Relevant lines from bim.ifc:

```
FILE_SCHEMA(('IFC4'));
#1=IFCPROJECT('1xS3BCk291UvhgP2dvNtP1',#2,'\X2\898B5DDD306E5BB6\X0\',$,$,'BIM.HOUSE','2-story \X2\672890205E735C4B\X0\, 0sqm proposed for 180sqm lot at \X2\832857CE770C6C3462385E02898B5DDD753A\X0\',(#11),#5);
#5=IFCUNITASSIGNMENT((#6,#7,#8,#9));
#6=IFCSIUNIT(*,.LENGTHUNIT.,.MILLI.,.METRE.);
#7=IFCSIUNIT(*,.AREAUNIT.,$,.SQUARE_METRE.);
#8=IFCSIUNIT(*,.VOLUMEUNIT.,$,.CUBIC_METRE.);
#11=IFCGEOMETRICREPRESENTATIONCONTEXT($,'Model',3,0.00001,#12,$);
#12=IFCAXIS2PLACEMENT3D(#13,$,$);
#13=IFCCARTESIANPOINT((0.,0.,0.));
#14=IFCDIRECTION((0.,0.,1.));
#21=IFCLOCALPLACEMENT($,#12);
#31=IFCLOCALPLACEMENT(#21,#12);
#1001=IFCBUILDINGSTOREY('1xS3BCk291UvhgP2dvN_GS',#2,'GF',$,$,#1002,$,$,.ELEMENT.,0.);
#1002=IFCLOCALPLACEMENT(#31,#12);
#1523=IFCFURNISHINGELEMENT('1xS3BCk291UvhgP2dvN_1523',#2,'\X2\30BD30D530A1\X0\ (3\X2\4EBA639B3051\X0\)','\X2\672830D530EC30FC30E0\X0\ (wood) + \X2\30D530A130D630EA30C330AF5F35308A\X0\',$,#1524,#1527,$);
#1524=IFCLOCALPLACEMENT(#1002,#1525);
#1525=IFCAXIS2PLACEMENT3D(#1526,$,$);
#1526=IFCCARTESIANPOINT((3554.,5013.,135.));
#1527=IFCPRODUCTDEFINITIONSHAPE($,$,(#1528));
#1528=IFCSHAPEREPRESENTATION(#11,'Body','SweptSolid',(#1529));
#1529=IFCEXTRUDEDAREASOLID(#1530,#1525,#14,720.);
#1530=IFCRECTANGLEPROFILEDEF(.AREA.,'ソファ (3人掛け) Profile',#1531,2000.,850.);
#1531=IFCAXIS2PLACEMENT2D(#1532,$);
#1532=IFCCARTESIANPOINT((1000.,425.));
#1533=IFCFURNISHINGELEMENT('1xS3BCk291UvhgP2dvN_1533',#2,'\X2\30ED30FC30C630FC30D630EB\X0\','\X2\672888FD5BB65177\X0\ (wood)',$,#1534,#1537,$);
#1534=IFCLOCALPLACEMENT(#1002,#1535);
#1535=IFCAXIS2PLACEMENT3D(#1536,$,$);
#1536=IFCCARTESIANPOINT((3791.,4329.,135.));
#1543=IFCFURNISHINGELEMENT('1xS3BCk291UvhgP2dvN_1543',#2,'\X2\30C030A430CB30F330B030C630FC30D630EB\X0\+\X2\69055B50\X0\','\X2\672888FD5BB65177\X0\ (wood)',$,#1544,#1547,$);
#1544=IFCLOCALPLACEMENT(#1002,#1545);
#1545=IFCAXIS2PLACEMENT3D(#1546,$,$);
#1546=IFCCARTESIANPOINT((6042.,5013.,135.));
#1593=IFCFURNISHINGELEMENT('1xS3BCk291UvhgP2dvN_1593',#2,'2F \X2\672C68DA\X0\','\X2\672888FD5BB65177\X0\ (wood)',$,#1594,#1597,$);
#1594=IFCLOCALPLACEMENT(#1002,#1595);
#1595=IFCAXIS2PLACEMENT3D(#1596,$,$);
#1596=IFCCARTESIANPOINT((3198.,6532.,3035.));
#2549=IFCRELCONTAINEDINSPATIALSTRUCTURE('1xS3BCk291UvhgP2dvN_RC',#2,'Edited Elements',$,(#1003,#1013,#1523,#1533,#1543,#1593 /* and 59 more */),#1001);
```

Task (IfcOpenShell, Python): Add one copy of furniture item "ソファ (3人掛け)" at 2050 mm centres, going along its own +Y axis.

```python
import ifcopenshell
import ifcopenshell.api.geometry
import ifcopenshell.api.root
import ifcopenshell.util.element
import ifcopenshell.util.placement
import ifcopenshell.util.unit

model = ifcopenshell.open("bim.ifc")
unit_scale = ifcopenshell.util.unit.calculate_unit_scale(model)


def reuse_history(source, copy):
    """copy_class also copies each property set's owner history, people and application; keep the originals."""
    for rel in copy.IsDefinedBy:
        if rel.is_a("IfcRelDefinesByProperties") and (history := rel.RelatingPropertyDefinition.OwnerHistory):
            rel.RelatingPropertyDefinition.OwnerHistory = source.OwnerHistory
            ifcopenshell.util.element.remove_deep2(model, history)


source = model.by_guid("1xS3BCk291UvhgP2dvN_1523")
base = ifcopenshell.util.placement.get_local_placement(source.ObjectPlacement)
step = base[:3, 1] * 2.05 / unit_scale

for i in range(1, 2):
    copy = ifcopenshell.api.root.copy_class(model, product=source)
    copy.Representation = ifcopenshell.util.element.copy_deep(
        model, source.Representation, exclude=["IfcGeometricRepresentationContext", "IfcRepresentationMap"]
    )
    reuse_history(source, copy)
    matrix = base.copy()
    matrix[:3, 3] += i * step
    print("added at", matrix[:3, 3].round(3) + 0.0)
    ifcopenshell.api.geometry.edit_object_placement(model, product=copy, matrix=matrix, is_si=False)

model.write("bim_v2.ifc")
```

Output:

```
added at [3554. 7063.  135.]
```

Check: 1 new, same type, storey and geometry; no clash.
